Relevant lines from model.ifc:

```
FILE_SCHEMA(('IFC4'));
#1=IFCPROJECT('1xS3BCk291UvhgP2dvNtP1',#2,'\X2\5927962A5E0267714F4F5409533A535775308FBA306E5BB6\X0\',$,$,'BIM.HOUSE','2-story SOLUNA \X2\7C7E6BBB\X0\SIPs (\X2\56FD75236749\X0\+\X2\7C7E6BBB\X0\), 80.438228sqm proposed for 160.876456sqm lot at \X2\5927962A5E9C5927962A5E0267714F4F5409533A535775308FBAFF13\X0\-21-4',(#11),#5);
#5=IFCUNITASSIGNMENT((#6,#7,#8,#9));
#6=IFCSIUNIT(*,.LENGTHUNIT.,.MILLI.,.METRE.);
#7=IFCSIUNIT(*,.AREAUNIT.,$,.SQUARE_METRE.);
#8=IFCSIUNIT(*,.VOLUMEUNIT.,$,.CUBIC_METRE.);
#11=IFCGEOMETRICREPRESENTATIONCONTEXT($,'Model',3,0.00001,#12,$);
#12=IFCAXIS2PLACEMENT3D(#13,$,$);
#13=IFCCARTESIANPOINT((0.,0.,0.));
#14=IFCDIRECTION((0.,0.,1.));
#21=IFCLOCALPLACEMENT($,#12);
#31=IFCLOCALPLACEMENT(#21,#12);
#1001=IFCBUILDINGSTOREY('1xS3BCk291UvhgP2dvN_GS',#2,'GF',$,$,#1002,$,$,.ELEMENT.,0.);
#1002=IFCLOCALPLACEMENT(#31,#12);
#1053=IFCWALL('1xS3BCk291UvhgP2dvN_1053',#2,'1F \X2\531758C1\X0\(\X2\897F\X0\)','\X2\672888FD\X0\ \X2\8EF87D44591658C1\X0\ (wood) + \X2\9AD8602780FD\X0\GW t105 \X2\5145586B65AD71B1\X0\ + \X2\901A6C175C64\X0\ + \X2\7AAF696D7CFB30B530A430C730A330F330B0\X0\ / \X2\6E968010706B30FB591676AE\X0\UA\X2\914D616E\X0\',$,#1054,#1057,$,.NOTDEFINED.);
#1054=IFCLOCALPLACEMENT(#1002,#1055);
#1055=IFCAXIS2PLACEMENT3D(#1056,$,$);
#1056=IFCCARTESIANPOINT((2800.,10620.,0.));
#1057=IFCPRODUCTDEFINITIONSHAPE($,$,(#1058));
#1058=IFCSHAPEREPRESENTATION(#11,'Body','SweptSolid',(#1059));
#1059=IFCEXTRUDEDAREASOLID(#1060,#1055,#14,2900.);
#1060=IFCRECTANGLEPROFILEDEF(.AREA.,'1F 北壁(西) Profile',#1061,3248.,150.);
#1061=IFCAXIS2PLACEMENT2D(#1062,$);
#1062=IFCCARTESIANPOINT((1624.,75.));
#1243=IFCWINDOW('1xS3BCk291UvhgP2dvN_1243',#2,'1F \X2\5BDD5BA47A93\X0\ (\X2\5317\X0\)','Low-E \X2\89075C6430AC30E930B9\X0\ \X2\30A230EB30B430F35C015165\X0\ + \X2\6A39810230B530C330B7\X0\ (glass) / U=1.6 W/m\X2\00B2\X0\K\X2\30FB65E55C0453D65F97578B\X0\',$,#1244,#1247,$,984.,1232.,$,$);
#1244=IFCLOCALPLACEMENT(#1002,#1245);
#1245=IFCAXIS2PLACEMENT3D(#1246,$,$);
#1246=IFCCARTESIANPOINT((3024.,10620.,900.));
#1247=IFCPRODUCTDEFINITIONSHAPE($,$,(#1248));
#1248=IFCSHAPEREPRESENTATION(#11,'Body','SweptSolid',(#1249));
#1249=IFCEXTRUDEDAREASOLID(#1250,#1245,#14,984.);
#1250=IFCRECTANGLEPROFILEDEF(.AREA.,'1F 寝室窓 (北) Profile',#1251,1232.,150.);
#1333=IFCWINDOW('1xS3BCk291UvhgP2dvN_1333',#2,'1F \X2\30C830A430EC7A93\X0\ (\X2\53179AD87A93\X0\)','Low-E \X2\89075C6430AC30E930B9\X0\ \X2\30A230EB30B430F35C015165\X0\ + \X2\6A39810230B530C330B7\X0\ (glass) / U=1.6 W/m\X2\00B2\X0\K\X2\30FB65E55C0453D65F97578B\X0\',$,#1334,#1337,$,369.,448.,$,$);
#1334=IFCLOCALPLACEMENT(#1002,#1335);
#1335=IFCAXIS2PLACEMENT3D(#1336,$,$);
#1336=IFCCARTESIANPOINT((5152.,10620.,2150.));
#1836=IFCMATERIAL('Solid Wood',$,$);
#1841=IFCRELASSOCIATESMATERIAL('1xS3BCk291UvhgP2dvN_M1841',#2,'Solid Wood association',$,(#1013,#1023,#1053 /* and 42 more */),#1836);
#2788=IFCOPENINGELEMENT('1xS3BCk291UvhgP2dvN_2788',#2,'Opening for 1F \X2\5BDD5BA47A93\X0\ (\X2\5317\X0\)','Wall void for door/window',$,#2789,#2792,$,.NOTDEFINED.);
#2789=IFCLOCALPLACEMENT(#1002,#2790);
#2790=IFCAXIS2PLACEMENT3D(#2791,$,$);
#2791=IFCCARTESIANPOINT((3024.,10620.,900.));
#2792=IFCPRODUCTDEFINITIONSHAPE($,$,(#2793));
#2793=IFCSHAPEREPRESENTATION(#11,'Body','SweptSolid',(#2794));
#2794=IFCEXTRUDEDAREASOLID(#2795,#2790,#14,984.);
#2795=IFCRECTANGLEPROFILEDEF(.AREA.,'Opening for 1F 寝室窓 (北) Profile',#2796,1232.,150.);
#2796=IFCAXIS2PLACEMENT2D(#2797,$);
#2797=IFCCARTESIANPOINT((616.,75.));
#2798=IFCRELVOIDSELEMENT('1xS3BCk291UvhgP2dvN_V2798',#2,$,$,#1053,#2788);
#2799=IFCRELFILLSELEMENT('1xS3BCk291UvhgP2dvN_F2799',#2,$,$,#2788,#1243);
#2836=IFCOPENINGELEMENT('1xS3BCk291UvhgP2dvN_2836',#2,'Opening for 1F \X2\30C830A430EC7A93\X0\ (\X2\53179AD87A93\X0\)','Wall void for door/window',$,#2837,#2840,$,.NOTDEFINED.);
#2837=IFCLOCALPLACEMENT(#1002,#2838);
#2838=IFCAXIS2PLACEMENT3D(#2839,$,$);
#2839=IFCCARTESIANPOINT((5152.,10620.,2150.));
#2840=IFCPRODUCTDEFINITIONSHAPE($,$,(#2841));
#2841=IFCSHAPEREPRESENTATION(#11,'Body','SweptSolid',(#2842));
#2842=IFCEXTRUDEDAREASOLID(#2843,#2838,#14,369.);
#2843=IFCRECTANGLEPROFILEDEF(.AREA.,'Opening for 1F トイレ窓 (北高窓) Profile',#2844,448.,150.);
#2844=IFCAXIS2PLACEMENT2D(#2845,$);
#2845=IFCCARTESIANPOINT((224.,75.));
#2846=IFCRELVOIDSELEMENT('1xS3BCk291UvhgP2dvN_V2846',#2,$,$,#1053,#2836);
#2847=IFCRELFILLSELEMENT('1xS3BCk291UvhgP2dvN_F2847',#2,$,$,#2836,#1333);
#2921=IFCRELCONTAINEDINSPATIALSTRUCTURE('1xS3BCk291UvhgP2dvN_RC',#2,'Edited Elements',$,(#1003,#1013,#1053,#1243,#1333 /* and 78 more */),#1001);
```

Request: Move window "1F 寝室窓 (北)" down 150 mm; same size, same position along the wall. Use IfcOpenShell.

```python
import numpy as np
import ifcopenshell
import ifcopenshell.api.geometry
import ifcopenshell.util.placement
import ifcopenshell.util.unit

model = ifcopenshell.open("model.ifc")
unit_scale = ifcopenshell.util.unit.calculate_unit_scale(model)

window = model.by_id(1243)
opening = window.FillsVoids[0].RelatingOpeningElement
dz = -0.15 / unit_scale

shift = np.array([0.0, 0.0, dz])
# The window is not placed relative to its opening, so move both.
for product in (opening, window):
    matrix = ifcopenshell.util.placement.get_local_placement(product.ObjectPlacement)
    matrix[:3, 3] += shift
    ifcopenshell.api.geometry.edit_object_placement(model, product=product, matrix=matrix, is_si=False)

print(f"moved by {dz * unit_scale:+.3f} m")

model.write("model_v2.ifc")
```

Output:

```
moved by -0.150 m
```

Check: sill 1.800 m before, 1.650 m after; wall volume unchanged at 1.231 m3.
